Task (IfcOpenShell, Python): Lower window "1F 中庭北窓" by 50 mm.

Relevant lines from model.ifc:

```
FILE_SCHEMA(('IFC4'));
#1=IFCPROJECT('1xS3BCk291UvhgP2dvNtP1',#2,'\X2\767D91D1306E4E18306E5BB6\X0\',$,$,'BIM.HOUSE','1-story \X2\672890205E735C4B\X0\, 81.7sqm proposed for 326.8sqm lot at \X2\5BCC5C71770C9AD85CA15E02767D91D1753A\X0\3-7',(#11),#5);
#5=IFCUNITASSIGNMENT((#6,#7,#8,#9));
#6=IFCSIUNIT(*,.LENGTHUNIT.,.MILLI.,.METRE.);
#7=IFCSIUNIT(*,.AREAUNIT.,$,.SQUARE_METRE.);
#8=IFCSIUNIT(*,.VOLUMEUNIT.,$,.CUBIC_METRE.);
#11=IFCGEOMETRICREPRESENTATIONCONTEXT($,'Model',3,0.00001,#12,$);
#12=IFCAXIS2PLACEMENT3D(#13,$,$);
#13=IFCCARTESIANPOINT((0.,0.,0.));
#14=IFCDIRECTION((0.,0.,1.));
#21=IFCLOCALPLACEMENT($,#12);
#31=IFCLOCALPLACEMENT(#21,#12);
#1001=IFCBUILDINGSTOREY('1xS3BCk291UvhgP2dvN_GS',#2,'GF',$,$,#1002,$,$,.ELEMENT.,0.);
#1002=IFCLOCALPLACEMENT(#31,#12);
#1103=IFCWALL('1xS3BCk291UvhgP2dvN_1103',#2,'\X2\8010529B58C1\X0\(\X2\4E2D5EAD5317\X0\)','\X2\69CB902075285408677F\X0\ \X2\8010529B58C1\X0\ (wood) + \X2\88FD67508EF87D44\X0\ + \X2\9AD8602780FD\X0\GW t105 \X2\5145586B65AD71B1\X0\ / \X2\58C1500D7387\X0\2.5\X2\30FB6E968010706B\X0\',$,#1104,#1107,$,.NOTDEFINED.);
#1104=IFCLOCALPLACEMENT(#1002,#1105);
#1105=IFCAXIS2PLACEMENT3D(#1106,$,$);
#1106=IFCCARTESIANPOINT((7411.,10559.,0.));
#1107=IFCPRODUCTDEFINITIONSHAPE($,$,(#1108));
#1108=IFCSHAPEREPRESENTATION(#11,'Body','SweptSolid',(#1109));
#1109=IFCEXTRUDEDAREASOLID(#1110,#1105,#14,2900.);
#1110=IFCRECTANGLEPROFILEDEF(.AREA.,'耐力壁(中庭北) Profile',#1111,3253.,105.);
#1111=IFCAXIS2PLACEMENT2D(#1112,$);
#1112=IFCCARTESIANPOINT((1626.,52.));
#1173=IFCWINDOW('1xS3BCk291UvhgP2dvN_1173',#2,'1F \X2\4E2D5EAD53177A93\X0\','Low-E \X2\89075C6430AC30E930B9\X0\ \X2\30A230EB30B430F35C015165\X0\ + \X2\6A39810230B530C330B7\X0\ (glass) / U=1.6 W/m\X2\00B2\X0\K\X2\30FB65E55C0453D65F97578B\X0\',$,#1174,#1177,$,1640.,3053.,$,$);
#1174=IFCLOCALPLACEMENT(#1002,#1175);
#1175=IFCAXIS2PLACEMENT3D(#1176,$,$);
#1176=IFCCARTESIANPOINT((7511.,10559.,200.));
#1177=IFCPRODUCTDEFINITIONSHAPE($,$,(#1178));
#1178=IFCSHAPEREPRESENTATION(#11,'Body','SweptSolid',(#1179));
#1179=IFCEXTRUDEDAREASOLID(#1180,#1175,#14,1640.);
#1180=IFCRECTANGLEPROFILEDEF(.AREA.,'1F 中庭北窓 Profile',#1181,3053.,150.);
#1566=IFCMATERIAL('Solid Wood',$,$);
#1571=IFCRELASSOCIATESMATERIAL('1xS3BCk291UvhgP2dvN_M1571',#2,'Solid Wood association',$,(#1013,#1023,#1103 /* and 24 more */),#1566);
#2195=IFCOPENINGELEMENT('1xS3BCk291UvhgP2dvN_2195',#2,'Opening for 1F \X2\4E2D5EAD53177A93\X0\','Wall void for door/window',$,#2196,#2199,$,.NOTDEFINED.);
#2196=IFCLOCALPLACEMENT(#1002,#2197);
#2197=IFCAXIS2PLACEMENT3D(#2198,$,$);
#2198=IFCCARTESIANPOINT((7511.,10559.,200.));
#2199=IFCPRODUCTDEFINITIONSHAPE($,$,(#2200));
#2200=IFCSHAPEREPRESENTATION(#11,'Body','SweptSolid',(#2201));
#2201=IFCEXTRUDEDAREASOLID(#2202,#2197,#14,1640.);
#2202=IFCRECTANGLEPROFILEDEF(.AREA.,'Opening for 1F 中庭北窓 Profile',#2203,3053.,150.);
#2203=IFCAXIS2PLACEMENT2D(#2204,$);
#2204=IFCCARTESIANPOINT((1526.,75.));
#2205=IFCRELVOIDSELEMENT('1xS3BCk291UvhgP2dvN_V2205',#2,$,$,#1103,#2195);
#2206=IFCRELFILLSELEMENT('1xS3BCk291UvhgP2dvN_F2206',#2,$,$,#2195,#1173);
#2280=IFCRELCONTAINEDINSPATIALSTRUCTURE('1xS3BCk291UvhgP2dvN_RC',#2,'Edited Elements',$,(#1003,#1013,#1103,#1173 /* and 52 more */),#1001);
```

```python
import numpy as np
import ifcopenshell
import ifcopenshell.api.geometry
import ifcopenshell.util.placement
import ifcopenshell.util.unit

model = ifcopenshell.open("model.ifc")
unit_scale = ifcopenshell.util.unit.calculate_unit_scale(model)

window = model.by_guid("1xS3BCk291UvhgP2dvN_1173")
opening = window.FillsVoids[0].RelatingOpeningElement
dz = -0.05 / unit_scale

shift = np.array([0.0, 0.0, dz])
# The window is not placed relative to its opening, so move both.
for product in (opening, window):
    matrix = ifcopenshell.util.placement.get_local_placement(product.ObjectPlacement)
    matrix[:3, 3] += shift
    ifcopenshell.api.geometry.edit_object_placement(model, product=product, matrix=matrix, is_si=False)

print(f"moved by {dz * unit_scale:+.3f} m")

model.write("model_v2.ifc")
```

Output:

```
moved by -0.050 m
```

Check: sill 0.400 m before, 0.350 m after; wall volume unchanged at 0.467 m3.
